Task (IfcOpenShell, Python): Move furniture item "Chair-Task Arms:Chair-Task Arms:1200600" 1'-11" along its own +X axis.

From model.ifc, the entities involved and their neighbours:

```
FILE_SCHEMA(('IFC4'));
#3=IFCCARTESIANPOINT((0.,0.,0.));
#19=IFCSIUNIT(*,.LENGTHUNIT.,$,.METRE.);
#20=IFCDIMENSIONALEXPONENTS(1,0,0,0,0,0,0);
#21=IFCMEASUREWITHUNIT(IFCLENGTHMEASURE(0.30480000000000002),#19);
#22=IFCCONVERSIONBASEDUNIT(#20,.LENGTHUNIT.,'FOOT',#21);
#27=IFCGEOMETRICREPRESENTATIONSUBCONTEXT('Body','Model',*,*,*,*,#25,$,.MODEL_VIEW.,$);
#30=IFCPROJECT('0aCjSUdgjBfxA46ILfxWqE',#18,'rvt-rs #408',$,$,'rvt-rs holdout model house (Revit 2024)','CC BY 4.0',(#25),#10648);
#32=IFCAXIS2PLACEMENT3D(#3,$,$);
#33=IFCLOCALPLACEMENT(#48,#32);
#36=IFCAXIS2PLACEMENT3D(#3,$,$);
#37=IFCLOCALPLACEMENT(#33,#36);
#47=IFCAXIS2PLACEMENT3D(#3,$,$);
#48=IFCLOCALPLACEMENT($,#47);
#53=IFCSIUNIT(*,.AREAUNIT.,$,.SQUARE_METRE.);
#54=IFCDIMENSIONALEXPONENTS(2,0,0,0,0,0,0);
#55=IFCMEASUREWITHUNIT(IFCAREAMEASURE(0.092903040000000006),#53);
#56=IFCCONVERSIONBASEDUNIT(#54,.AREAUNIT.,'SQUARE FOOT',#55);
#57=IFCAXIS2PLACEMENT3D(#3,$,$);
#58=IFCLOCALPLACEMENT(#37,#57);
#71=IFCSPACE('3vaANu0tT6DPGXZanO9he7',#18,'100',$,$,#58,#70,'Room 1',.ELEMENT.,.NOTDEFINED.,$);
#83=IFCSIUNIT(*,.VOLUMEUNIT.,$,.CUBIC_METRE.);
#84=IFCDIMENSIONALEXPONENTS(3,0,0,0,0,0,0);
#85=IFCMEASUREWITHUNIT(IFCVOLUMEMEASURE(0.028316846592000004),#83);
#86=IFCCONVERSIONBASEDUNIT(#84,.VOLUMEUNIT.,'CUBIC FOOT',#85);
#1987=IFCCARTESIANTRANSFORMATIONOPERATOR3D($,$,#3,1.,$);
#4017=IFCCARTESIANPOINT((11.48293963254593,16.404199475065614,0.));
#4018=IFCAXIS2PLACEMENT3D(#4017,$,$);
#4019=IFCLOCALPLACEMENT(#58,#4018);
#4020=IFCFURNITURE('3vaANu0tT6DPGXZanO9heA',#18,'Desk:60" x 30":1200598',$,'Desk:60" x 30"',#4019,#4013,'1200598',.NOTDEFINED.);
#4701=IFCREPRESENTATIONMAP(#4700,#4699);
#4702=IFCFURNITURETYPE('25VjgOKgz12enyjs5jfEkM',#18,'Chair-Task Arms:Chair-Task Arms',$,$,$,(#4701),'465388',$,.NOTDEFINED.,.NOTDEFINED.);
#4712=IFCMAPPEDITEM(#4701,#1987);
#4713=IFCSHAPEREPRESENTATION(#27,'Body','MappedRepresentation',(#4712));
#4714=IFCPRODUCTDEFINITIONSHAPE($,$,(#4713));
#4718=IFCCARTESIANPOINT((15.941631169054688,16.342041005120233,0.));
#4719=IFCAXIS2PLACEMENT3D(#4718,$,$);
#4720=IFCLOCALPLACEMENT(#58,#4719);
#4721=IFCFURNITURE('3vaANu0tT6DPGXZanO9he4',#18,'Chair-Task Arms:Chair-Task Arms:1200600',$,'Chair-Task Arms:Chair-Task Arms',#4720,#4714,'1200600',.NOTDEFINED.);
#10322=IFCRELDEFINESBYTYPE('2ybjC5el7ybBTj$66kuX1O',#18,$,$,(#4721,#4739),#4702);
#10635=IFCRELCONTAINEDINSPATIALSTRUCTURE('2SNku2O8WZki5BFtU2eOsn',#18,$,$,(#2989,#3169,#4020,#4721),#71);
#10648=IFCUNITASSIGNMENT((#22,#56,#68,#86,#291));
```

```python
import ifcopenshell
import ifcopenshell.api.geometry
import ifcopenshell.util.placement
import ifcopenshell.util.unit

model = ifcopenshell.open("model.ifc")
unit_scale = ifcopenshell.util.unit.calculate_unit_scale(model)

item = model.by_id(4721)
matrix = ifcopenshell.util.placement.get_local_placement(item.ObjectPlacement)
matrix[:3, 3] += matrix[:3, 0] * 23 * 0.0254 / unit_scale
ifcopenshell.api.geometry.edit_object_placement(model, product=item, matrix=matrix, is_si=False)

print(ifcopenshell.util.placement.get_local_placement(item.ObjectPlacement).round(3) + 0.0)

model.write("model_rev.ifc")
```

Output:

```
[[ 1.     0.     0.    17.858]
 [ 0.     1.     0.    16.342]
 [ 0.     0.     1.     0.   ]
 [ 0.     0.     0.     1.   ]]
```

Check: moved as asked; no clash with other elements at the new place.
